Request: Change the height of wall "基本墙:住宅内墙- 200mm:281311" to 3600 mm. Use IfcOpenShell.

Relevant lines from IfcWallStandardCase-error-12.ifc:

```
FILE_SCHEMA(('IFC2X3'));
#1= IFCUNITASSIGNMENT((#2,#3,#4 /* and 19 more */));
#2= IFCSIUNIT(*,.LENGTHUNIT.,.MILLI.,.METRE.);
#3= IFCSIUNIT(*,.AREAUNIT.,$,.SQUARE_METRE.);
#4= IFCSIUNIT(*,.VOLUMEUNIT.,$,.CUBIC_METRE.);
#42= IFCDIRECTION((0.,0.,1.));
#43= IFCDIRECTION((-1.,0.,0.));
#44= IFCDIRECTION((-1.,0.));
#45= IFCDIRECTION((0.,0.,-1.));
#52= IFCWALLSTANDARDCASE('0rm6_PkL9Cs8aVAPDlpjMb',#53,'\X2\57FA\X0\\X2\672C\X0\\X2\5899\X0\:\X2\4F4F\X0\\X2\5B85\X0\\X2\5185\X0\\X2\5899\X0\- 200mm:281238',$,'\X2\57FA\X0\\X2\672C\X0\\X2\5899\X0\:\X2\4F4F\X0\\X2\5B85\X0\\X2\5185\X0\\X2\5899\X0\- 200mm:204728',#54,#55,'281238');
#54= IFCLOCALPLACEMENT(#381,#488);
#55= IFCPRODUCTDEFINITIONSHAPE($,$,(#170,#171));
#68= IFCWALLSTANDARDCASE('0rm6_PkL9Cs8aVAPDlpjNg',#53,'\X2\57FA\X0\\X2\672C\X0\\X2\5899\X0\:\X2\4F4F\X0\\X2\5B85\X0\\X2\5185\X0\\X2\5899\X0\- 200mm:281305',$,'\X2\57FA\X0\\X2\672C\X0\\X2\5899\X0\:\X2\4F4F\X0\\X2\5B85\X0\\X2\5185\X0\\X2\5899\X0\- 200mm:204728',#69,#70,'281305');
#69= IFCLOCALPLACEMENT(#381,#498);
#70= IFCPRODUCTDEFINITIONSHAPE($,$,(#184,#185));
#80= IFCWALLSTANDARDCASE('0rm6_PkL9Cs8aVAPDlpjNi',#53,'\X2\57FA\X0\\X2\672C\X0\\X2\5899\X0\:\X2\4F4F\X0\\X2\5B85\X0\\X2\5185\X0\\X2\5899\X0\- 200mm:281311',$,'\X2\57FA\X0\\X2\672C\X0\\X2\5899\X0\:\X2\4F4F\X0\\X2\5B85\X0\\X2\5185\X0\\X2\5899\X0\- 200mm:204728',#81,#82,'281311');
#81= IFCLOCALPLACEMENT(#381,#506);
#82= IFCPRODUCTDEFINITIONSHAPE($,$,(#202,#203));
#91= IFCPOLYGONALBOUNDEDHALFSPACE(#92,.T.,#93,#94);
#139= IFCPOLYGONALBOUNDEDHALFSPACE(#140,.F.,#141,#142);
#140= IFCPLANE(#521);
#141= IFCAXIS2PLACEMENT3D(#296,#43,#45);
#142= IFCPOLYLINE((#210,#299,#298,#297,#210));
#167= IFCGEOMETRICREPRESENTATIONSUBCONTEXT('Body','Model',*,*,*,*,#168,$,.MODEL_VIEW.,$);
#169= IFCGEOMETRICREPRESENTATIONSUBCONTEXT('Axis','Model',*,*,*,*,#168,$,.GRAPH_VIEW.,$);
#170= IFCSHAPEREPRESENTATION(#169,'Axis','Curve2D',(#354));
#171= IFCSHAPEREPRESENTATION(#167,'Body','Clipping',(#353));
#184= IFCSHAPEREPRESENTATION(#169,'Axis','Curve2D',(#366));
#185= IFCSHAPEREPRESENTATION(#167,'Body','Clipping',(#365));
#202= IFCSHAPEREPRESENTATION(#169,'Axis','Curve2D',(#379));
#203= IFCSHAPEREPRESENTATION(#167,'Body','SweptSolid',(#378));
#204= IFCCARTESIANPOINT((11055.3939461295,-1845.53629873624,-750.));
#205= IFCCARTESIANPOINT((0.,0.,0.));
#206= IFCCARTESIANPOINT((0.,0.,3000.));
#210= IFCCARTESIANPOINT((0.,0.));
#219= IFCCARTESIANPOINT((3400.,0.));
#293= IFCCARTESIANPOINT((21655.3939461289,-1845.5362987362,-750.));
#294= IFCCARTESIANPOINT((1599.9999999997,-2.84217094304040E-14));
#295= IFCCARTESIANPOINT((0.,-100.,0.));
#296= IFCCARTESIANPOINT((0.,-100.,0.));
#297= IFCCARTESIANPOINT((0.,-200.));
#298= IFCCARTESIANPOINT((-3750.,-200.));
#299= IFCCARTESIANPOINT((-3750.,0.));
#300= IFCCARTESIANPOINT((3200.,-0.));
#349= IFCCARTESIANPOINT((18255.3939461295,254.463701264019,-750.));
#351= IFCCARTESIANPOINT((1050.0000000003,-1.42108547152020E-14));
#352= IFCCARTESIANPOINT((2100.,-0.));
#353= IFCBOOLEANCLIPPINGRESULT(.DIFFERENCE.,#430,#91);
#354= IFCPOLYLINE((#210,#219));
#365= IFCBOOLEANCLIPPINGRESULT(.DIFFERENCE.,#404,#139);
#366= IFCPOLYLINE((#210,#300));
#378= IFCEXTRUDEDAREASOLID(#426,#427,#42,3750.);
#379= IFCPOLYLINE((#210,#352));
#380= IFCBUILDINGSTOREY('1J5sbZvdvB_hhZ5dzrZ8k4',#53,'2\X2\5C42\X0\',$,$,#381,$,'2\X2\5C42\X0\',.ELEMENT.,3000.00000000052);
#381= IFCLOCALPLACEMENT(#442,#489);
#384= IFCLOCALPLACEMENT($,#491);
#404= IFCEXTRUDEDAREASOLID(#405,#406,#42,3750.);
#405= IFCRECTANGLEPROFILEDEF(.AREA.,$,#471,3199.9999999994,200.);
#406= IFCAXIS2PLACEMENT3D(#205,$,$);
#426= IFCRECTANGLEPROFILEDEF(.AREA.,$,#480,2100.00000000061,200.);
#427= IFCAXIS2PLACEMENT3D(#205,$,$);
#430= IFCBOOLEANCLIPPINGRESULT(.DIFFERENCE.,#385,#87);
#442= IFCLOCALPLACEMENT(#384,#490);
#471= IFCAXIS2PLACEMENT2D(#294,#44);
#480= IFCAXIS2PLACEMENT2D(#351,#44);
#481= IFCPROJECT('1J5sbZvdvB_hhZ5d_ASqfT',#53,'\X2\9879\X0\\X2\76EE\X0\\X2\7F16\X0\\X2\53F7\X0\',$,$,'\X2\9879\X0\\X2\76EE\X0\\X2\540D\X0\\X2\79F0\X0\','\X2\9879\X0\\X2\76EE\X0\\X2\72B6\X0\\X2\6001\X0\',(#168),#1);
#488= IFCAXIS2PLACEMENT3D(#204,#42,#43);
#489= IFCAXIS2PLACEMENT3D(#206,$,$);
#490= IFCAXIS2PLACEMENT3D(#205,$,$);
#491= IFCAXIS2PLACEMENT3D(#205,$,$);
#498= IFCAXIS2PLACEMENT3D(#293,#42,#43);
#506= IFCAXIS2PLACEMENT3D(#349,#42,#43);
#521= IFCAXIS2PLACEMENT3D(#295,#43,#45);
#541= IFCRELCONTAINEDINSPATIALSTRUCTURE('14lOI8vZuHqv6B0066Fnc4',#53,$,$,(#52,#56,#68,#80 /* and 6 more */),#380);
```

```python
import ifcopenshell
import ifcopenshell.geom
import ifcopenshell.util.representation
import ifcopenshell.util.shape

model = ifcopenshell.open("IfcWallStandardCase-error-12.ifc")
settings = ifcopenshell.geom.settings()


def volume(element):
    """Net volume in cubic metres, openings subtracted."""
    shape = ifcopenshell.geom.create_shape(settings, element)
    return ifcopenshell.util.shape.get_volume(shape.geometry)


wall = model.by_guid("0rm6_PkL9Cs8aVAPDlpjNi")
before = volume(wall)

body = ifcopenshell.util.representation.get_representation(wall, "Model", "Body")
solid = body.Items[0]
old_height = solid.Depth
solid.Depth = 3600.0
after = volume(wall)

print(f"height {old_height:g} -> {solid.Depth:g}, volume {before:.3f} -> {after:.3f} m3")

model.write("IfcWallStandardCase-error-12-out.ifc")
```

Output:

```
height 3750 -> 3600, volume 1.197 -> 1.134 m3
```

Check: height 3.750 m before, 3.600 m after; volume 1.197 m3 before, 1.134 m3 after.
